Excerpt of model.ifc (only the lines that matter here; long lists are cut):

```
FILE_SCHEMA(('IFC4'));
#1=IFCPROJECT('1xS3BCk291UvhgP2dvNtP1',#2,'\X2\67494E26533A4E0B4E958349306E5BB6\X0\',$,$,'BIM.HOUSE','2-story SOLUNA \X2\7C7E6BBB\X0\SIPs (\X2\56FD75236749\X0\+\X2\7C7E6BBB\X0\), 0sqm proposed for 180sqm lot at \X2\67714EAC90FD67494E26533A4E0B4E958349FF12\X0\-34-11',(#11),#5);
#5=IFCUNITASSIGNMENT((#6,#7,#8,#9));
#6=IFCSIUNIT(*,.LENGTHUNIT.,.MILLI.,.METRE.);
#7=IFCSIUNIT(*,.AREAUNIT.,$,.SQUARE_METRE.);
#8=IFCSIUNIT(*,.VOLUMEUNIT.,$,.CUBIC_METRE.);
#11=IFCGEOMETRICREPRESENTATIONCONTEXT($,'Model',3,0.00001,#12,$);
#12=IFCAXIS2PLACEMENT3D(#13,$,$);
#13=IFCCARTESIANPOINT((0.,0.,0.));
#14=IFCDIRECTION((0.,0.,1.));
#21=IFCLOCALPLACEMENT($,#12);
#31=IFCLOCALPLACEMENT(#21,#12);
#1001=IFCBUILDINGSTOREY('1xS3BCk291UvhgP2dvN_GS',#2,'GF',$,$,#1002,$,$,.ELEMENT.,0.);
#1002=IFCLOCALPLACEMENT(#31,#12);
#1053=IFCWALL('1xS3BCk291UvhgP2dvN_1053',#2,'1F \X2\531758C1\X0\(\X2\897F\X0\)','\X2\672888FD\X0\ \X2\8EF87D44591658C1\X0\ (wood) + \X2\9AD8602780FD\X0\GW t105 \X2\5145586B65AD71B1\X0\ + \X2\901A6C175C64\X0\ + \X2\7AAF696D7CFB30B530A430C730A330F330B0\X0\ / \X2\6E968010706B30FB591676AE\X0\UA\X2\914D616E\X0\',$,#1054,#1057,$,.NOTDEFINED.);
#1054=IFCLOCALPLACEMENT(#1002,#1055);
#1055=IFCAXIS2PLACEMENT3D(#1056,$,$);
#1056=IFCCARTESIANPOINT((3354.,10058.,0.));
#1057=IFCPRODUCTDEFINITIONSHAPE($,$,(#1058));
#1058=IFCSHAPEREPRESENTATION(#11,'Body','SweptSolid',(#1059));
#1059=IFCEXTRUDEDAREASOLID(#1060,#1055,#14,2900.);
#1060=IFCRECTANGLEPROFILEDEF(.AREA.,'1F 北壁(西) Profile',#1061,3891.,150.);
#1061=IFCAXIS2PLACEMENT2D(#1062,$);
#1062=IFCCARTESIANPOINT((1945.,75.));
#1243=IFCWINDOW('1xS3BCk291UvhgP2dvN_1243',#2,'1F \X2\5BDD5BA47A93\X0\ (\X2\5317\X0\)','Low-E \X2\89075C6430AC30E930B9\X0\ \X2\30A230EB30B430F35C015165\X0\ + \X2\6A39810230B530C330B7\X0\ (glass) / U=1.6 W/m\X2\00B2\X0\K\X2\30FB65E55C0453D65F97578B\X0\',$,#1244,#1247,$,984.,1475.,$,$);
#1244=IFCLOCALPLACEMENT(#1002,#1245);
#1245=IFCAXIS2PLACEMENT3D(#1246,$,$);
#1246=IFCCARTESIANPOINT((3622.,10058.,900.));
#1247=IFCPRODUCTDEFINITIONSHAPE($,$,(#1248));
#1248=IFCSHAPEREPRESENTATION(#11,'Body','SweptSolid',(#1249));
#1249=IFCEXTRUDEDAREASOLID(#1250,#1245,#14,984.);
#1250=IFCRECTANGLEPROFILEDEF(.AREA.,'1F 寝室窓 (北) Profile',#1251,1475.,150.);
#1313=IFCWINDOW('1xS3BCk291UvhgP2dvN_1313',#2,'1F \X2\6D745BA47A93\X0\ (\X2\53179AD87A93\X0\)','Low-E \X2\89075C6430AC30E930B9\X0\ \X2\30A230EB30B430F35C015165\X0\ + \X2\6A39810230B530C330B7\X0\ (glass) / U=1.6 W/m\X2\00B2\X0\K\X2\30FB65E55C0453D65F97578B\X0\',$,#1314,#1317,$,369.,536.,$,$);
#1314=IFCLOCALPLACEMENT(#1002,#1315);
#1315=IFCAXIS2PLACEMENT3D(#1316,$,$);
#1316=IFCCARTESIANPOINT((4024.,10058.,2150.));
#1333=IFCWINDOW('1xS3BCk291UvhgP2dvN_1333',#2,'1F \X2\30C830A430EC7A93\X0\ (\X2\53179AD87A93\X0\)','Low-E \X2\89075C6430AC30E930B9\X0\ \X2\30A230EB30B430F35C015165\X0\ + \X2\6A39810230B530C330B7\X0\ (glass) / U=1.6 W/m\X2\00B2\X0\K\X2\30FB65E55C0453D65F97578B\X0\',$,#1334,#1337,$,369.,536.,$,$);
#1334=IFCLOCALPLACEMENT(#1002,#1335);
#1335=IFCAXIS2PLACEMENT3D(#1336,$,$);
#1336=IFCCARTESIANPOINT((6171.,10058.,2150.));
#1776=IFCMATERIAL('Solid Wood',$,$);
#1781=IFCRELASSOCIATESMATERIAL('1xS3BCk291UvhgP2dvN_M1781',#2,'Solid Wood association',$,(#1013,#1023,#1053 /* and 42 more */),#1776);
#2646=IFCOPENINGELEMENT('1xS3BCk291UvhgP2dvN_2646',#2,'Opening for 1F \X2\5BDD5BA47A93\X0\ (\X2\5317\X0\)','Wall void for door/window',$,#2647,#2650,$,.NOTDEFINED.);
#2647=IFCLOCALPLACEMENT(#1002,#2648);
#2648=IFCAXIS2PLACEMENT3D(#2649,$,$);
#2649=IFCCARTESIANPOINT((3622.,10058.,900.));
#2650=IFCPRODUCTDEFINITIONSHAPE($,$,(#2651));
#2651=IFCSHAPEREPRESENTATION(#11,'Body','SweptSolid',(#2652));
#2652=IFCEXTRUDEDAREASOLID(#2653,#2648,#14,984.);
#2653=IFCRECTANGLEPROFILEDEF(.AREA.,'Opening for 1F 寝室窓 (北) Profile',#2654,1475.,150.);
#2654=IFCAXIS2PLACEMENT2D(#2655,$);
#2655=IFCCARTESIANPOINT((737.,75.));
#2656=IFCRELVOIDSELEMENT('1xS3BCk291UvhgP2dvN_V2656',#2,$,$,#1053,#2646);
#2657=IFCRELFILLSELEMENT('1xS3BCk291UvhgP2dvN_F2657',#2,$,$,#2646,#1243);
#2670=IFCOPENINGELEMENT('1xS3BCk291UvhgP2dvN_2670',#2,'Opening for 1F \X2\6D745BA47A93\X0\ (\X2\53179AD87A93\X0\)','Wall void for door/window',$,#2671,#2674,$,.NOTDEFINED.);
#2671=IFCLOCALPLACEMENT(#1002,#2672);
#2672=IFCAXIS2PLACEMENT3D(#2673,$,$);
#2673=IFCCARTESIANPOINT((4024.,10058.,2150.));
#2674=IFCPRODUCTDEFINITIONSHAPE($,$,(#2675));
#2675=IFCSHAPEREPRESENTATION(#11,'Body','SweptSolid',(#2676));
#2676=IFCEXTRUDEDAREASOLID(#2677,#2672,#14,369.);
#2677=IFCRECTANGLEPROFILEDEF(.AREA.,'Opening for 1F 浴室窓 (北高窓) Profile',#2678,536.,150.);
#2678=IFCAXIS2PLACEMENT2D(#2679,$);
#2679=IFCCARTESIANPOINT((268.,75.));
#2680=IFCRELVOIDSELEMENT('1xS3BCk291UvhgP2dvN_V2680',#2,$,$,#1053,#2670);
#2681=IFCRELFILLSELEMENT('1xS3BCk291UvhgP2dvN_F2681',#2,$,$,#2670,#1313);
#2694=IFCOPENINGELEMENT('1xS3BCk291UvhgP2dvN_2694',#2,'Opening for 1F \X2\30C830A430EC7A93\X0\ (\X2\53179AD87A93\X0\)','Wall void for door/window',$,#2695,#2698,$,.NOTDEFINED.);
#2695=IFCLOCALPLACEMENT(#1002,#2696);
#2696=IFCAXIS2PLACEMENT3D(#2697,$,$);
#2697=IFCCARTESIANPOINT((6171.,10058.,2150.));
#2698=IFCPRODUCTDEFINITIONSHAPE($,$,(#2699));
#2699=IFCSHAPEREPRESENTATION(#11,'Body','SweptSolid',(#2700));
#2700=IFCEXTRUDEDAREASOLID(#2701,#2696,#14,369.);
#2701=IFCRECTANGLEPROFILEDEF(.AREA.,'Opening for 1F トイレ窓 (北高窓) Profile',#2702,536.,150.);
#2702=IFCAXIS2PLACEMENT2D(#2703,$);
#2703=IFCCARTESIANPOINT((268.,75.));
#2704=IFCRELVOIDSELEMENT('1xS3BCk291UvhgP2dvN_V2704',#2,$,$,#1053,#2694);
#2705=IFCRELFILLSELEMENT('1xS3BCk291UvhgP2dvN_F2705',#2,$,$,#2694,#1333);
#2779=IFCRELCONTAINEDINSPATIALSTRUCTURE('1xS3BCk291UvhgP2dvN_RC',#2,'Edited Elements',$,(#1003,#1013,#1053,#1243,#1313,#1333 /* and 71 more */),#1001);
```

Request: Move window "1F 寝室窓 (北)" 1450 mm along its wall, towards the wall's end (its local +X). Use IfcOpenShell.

```python
import ifcopenshell
import ifcopenshell.api.geometry
import ifcopenshell.util.placement

model = ifcopenshell.open("model.ifc")

window = model.by_id(1243)
opening = window.FillsVoids[0].RelatingOpeningElement
wall = opening.VoidsElements[0].RelatingBuildingElement

wall_matrix = ifcopenshell.util.placement.get_local_placement(wall.ObjectPlacement)
shift = wall_matrix[:3, 0] * 1450.0
before = ifcopenshell.util.placement.get_local_placement(window.ObjectPlacement)[:3, 3].copy()

# The window is not placed relative to its opening, so move both.
for product in (opening, window):
    matrix = ifcopenshell.util.placement.get_local_placement(product.ObjectPlacement)
    matrix[:3, 3] += shift
    ifcopenshell.api.geometry.edit_object_placement(model, product=product, matrix=matrix, is_si=False)

after = ifcopenshell.util.placement.get_local_placement(window.ObjectPlacement)[:3, 3]
print("window moved by", (after - before).round(3) + 0.0)

model.write("model-out.ifc")
```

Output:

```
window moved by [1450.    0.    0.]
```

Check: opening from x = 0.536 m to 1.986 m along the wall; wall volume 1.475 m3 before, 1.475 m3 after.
